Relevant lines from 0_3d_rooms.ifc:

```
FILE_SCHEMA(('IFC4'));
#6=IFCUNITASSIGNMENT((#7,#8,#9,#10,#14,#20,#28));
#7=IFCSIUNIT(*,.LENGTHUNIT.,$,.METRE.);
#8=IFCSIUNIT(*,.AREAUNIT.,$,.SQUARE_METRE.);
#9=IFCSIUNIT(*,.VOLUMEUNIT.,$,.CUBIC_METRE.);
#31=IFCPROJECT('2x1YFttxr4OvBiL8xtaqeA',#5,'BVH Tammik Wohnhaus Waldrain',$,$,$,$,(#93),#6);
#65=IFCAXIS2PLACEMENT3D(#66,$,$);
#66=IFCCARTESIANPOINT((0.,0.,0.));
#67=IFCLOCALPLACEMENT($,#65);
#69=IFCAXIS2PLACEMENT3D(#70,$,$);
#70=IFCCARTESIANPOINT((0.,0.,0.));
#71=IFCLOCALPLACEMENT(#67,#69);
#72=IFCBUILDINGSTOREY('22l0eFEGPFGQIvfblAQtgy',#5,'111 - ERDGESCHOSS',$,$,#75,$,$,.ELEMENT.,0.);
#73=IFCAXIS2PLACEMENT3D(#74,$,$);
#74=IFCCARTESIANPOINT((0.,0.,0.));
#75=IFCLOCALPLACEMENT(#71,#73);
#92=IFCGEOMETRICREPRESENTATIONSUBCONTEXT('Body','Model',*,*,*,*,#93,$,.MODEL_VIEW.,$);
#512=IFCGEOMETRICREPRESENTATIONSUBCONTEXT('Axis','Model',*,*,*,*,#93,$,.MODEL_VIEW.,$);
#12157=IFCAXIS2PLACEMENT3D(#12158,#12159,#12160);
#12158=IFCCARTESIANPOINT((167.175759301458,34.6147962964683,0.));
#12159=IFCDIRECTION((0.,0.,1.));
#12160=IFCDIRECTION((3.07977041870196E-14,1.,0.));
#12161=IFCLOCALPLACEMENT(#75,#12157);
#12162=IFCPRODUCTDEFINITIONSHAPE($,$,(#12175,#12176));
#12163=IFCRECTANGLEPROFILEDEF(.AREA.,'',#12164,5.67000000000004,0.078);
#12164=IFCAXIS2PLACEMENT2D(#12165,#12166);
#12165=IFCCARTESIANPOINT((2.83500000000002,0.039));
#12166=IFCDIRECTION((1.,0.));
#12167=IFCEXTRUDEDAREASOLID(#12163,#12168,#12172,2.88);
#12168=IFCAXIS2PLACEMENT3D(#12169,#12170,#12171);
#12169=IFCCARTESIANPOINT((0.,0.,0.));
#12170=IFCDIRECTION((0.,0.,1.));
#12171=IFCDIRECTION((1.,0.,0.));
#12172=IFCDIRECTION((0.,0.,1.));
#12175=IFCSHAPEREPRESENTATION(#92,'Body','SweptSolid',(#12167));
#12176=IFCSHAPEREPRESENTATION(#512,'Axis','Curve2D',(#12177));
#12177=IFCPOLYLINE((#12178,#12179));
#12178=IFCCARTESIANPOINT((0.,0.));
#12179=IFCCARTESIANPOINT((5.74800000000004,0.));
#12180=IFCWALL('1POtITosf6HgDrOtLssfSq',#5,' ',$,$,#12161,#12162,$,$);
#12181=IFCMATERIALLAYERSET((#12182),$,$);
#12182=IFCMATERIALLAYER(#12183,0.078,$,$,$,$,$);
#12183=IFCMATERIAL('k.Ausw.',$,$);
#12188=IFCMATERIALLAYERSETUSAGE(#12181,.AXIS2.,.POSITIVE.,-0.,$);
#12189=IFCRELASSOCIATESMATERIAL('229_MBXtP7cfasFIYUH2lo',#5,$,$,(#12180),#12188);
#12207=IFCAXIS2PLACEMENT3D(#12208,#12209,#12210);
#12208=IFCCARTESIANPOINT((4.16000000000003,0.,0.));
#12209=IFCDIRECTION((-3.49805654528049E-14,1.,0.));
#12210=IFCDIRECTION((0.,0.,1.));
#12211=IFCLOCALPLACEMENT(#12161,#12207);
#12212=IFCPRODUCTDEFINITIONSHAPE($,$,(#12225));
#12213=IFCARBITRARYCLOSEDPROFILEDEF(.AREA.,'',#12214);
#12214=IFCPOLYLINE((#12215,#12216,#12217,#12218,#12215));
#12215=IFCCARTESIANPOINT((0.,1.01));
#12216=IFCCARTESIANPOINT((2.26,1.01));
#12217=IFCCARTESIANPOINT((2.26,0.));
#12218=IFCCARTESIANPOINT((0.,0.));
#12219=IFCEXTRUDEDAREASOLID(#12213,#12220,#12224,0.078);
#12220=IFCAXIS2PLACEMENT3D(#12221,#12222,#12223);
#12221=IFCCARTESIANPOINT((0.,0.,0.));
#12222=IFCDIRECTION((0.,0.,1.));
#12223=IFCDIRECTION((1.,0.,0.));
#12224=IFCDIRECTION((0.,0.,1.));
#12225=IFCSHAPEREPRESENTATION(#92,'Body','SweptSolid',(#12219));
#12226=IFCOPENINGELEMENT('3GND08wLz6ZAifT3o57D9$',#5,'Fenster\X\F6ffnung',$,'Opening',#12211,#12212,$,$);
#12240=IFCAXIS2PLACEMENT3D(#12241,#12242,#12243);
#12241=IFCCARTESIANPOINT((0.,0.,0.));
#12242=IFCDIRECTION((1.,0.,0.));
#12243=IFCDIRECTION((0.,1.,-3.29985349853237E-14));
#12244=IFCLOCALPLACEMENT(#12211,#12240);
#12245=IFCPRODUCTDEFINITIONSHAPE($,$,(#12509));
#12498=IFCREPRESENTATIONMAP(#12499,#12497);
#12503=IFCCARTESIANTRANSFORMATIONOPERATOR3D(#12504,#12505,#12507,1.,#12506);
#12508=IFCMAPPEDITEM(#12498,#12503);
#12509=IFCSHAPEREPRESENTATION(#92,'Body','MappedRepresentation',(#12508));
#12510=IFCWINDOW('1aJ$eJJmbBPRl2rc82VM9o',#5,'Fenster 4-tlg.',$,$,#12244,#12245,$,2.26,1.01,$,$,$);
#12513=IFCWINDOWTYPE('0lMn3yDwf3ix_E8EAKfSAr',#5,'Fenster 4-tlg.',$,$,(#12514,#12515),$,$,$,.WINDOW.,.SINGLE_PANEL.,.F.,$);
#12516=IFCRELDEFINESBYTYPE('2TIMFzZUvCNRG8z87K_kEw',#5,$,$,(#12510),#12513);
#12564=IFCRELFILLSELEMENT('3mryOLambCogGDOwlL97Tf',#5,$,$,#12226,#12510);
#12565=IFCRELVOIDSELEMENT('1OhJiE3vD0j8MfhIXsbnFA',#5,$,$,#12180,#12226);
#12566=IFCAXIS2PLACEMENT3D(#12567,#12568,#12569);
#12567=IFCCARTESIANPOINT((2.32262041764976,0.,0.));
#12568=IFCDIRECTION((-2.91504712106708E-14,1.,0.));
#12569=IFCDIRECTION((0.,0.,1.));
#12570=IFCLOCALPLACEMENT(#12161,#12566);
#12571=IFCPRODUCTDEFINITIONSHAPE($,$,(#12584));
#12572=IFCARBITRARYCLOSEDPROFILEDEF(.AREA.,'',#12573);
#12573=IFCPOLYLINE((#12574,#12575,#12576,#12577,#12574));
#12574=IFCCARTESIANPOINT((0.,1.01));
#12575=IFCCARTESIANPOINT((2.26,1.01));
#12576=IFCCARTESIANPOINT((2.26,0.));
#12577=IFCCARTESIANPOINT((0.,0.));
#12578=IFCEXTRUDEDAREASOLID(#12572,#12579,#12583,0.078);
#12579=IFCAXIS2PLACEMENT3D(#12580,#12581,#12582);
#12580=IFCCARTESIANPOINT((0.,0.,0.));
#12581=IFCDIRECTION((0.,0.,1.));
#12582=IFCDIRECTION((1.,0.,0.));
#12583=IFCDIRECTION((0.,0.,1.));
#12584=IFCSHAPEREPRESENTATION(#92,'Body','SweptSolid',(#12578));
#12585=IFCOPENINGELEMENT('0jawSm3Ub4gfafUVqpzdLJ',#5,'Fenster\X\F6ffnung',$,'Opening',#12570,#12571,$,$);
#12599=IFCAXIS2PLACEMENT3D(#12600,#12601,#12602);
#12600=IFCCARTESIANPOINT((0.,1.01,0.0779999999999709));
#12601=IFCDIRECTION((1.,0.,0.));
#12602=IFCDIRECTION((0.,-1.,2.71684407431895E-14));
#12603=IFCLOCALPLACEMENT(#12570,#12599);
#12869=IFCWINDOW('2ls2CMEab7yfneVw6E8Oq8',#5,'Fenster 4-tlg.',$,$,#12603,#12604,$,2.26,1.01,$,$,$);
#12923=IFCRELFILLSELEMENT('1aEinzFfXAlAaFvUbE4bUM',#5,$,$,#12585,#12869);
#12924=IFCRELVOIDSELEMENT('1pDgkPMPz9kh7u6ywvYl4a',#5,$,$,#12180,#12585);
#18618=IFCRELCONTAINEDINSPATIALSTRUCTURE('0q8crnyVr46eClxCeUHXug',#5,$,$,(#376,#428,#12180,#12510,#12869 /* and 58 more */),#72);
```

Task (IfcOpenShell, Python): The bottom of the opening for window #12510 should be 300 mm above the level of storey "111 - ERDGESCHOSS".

```python
import numpy as np
import ifcopenshell
import ifcopenshell.api.geometry
import ifcopenshell.geom
import ifcopenshell.util.element
import ifcopenshell.util.placement
import ifcopenshell.util.shape
import ifcopenshell.util.unit

model = ifcopenshell.open("0_3d_rooms.ifc")
unit_scale = ifcopenshell.util.unit.calculate_unit_scale(model)

window = model.by_id(12510)
opening = window.FillsVoids[0].RelatingOpeningElement
storey = ifcopenshell.util.element.get_container(window, ifc_class="IfcBuildingStorey")
level = ifcopenshell.util.placement.get_local_placement(storey.ObjectPlacement)[2, 3]

# The opening's origin need not be at the sill, so measure its lowest point.
shape = ifcopenshell.geom.create_shape(ifcopenshell.geom.settings(), opening)
bottom = ifcopenshell.util.shape.get_shape_bottom_elevation(shape, shape.geometry) / unit_scale
dz = level + 0.3 - bottom

shift = np.array([0.0, 0.0, dz])
# The window is placed relative to its opening, so it follows when the opening moves.
matrix = ifcopenshell.util.placement.get_local_placement(opening.ObjectPlacement)
matrix[:3, 3] += shift
ifcopenshell.api.geometry.edit_object_placement(
    model, product=opening, matrix=matrix, is_si=False, should_transform_children=True
)

print(f"moved by {dz * unit_scale:+.3f} m")

model.write("0_3d_rooms_edited.ifc")
```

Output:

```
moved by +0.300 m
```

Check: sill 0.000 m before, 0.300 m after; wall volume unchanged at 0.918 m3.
